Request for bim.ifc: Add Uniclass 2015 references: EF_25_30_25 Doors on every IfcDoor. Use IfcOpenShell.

First a look at what the model holds.

```python
import ifcopenshell

model = ifcopenshell.open("bim.ifc")
print(model.schema)
print("classifications:", [c.Name for c in model.by_type("IfcClassification")])
for ifc_class in ("IfcDoor", "IfcRoof", "IfcStair", "IfcWall", "IfcWindow"):
    print(ifc_class, len(model.by_type(ifc_class)))
```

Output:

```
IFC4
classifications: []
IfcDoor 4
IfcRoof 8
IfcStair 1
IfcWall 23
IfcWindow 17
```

```python
import ifcopenshell
import ifcopenshell.api.classification

model = ifcopenshell.open("bim.ifc")

system = ifcopenshell.api.classification.add_classification(model, classification="Uniclass 2015")

codes = {
    "IfcDoor": ("EF_25_30_25", "Doors"),
}
for ifc_class, (code, name) in codes.items():
    products = model.by_type(ifc_class)
    ifcopenshell.api.classification.add_reference(
        model, products=products, classification=system, identification=code, name=name
    )
    print(code, len(products))

model.write("bim-out.ifc")
```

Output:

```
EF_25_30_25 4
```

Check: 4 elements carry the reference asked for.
